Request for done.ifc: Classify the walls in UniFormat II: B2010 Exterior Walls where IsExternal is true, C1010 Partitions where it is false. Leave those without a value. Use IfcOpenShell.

First a look at what the model holds.

```python
import ifcopenshell
import ifcopenshell.util.element

model = ifcopenshell.open("done.ifc")
print(model.schema)
print("classifications:", [c.Name for c in model.by_type("IfcClassification")])
values = [ifcopenshell.util.element.get_pset(e, "Pset_WallCommon", "IsExternal") for e in model.by_type("IfcWall")]
for value in (True, False, None):
    print("IsExternal", value, values.count(value))
```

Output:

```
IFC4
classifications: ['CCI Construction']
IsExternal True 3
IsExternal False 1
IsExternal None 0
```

```python
import ifcopenshell
import ifcopenshell.api.classification
import ifcopenshell.util.element

model = ifcopenshell.open("done.ifc")

system = ifcopenshell.api.classification.add_classification(model, classification="UniFormat II")

walls = model.by_type("IfcWall")
external = {e: ifcopenshell.util.element.get_pset(e, "Pset_WallCommon", "IsExternal") for e in walls}
for flag, code, name in ((True, "B2010", "Exterior Walls"), (False, "C1010", "Partitions")):
    products = [e for e in walls if external[e] is flag]
    ifcopenshell.api.classification.add_reference(
        model, products=products, classification=system, identification=code, name=name
    )
    print(code, len(products))

model.write("done_v2.ifc")
```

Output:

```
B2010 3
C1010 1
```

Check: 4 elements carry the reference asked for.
